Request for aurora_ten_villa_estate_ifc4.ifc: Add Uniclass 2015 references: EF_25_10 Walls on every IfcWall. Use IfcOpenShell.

First a look at what the model holds.

```python
import ifcopenshell

model = ifcopenshell.open("aurora_ten_villa_estate_ifc4.ifc")
print(model.schema)
print("classifications:", [c.Name for c in model.by_type("IfcClassification")])
for ifc_class in ("IfcDoor", "IfcRoof", "IfcStair", "IfcWall", "IfcWindow"):
    print(ifc_class, len(model.by_type(ifc_class)))
```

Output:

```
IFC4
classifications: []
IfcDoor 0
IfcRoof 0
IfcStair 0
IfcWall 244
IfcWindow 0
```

```python
import ifcopenshell
import ifcopenshell.api.classification

model = ifcopenshell.open("aurora_ten_villa_estate_ifc4.ifc")

system = ifcopenshell.api.classification.add_classification(model, classification="Uniclass 2015")

codes = {
    "IfcWall": ("EF_25_10", "Walls"),
}
for ifc_class, (code, name) in codes.items():
    products = model.by_type(ifc_class)
    ifcopenshell.api.classification.add_reference(
        model, products=products, classification=system, identification=code, name=name
    )
    print(code, len(products))

model.write("aurora_ten_villa_estate_ifc4_updated.ifc")
```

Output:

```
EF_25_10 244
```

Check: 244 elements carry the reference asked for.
